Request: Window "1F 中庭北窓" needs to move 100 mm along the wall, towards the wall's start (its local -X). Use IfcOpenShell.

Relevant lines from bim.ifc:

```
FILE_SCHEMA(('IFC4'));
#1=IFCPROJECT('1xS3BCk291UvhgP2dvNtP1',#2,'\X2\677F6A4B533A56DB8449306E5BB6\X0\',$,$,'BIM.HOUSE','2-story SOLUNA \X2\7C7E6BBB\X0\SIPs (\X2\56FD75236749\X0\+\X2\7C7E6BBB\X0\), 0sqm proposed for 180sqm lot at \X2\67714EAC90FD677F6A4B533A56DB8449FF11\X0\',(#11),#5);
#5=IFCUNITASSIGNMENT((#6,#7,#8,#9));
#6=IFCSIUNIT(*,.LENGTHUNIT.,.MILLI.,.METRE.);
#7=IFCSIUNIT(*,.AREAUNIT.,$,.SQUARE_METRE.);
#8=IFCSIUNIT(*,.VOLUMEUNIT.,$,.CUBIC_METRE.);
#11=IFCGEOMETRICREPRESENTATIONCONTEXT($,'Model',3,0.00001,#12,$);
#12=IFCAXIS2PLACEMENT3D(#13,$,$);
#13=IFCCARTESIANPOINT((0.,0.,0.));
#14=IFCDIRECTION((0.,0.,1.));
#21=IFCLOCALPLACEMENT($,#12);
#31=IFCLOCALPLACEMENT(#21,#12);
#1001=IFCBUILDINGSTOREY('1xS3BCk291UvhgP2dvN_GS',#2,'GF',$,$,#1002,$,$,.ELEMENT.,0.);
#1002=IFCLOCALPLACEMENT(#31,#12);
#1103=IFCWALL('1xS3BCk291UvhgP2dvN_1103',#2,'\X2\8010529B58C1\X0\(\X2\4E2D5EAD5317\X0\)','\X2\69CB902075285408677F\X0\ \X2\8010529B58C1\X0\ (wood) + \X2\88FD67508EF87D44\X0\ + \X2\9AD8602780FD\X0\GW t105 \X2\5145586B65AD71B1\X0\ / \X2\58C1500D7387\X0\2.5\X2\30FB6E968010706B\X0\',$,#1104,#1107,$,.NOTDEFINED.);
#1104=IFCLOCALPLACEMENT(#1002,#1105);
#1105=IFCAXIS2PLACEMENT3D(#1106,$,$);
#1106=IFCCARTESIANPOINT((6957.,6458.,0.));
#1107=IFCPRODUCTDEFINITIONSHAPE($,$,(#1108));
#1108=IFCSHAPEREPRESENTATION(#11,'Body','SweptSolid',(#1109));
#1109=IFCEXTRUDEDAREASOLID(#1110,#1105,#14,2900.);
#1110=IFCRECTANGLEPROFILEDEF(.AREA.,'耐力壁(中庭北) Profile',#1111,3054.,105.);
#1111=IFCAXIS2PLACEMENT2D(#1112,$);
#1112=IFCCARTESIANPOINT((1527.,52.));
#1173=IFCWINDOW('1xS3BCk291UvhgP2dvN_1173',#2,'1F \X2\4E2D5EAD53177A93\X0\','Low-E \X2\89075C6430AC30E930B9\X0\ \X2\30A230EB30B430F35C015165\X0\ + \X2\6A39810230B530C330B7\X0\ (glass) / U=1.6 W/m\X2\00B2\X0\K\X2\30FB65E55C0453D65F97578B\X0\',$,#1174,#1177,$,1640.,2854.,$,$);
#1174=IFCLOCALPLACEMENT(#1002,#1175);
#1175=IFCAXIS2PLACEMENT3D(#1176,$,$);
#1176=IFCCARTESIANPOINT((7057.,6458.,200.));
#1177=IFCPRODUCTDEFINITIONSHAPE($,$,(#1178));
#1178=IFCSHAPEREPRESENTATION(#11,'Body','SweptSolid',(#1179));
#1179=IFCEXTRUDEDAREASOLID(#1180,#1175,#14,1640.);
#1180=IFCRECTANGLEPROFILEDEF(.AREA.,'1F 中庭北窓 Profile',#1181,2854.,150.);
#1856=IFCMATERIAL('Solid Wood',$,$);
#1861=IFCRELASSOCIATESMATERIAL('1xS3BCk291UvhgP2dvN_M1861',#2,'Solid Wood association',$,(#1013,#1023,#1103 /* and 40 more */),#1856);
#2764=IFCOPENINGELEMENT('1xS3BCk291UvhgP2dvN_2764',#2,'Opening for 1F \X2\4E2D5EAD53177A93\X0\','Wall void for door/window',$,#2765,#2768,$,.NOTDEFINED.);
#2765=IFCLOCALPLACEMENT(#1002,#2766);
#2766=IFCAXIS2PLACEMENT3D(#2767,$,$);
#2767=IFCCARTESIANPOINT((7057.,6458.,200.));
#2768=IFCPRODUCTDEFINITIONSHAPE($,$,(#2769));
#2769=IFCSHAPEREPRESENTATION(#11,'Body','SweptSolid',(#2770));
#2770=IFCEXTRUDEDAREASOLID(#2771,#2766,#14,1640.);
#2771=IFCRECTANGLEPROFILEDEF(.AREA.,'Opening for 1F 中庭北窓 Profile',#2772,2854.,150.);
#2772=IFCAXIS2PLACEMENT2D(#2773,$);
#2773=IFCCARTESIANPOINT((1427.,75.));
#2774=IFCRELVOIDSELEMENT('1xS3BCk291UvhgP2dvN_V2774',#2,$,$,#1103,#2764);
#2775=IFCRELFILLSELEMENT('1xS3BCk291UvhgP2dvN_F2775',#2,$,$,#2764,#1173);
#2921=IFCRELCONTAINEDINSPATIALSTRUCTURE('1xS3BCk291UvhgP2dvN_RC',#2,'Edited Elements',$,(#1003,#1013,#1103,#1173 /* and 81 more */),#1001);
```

```python
import ifcopenshell
import ifcopenshell.api.geometry
import ifcopenshell.util.placement

model = ifcopenshell.open("bim.ifc")

window = model.by_id(1173)
opening = window.FillsVoids[0].RelatingOpeningElement
wall = opening.VoidsElements[0].RelatingBuildingElement

wall_matrix = ifcopenshell.util.placement.get_local_placement(wall.ObjectPlacement)
shift = wall_matrix[:3, 0] * -100.0
before = ifcopenshell.util.placement.get_local_placement(window.ObjectPlacement)[:3, 3].copy()

# The window is not placed relative to its opening, so move both.
for product in (opening, window):
    matrix = ifcopenshell.util.placement.get_local_placement(product.ObjectPlacement)
    matrix[:3, 3] += shift
    ifcopenshell.api.geometry.edit_object_placement(model, product=product, matrix=matrix, is_si=False)

after = ifcopenshell.util.placement.get_local_placement(window.ObjectPlacement)[:3, 3]
print("window moved by", (after - before).round(3) + 0.0)

model.write("bim_rev.ifc")
```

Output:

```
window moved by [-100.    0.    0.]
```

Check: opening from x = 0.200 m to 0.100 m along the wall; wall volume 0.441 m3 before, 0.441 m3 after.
